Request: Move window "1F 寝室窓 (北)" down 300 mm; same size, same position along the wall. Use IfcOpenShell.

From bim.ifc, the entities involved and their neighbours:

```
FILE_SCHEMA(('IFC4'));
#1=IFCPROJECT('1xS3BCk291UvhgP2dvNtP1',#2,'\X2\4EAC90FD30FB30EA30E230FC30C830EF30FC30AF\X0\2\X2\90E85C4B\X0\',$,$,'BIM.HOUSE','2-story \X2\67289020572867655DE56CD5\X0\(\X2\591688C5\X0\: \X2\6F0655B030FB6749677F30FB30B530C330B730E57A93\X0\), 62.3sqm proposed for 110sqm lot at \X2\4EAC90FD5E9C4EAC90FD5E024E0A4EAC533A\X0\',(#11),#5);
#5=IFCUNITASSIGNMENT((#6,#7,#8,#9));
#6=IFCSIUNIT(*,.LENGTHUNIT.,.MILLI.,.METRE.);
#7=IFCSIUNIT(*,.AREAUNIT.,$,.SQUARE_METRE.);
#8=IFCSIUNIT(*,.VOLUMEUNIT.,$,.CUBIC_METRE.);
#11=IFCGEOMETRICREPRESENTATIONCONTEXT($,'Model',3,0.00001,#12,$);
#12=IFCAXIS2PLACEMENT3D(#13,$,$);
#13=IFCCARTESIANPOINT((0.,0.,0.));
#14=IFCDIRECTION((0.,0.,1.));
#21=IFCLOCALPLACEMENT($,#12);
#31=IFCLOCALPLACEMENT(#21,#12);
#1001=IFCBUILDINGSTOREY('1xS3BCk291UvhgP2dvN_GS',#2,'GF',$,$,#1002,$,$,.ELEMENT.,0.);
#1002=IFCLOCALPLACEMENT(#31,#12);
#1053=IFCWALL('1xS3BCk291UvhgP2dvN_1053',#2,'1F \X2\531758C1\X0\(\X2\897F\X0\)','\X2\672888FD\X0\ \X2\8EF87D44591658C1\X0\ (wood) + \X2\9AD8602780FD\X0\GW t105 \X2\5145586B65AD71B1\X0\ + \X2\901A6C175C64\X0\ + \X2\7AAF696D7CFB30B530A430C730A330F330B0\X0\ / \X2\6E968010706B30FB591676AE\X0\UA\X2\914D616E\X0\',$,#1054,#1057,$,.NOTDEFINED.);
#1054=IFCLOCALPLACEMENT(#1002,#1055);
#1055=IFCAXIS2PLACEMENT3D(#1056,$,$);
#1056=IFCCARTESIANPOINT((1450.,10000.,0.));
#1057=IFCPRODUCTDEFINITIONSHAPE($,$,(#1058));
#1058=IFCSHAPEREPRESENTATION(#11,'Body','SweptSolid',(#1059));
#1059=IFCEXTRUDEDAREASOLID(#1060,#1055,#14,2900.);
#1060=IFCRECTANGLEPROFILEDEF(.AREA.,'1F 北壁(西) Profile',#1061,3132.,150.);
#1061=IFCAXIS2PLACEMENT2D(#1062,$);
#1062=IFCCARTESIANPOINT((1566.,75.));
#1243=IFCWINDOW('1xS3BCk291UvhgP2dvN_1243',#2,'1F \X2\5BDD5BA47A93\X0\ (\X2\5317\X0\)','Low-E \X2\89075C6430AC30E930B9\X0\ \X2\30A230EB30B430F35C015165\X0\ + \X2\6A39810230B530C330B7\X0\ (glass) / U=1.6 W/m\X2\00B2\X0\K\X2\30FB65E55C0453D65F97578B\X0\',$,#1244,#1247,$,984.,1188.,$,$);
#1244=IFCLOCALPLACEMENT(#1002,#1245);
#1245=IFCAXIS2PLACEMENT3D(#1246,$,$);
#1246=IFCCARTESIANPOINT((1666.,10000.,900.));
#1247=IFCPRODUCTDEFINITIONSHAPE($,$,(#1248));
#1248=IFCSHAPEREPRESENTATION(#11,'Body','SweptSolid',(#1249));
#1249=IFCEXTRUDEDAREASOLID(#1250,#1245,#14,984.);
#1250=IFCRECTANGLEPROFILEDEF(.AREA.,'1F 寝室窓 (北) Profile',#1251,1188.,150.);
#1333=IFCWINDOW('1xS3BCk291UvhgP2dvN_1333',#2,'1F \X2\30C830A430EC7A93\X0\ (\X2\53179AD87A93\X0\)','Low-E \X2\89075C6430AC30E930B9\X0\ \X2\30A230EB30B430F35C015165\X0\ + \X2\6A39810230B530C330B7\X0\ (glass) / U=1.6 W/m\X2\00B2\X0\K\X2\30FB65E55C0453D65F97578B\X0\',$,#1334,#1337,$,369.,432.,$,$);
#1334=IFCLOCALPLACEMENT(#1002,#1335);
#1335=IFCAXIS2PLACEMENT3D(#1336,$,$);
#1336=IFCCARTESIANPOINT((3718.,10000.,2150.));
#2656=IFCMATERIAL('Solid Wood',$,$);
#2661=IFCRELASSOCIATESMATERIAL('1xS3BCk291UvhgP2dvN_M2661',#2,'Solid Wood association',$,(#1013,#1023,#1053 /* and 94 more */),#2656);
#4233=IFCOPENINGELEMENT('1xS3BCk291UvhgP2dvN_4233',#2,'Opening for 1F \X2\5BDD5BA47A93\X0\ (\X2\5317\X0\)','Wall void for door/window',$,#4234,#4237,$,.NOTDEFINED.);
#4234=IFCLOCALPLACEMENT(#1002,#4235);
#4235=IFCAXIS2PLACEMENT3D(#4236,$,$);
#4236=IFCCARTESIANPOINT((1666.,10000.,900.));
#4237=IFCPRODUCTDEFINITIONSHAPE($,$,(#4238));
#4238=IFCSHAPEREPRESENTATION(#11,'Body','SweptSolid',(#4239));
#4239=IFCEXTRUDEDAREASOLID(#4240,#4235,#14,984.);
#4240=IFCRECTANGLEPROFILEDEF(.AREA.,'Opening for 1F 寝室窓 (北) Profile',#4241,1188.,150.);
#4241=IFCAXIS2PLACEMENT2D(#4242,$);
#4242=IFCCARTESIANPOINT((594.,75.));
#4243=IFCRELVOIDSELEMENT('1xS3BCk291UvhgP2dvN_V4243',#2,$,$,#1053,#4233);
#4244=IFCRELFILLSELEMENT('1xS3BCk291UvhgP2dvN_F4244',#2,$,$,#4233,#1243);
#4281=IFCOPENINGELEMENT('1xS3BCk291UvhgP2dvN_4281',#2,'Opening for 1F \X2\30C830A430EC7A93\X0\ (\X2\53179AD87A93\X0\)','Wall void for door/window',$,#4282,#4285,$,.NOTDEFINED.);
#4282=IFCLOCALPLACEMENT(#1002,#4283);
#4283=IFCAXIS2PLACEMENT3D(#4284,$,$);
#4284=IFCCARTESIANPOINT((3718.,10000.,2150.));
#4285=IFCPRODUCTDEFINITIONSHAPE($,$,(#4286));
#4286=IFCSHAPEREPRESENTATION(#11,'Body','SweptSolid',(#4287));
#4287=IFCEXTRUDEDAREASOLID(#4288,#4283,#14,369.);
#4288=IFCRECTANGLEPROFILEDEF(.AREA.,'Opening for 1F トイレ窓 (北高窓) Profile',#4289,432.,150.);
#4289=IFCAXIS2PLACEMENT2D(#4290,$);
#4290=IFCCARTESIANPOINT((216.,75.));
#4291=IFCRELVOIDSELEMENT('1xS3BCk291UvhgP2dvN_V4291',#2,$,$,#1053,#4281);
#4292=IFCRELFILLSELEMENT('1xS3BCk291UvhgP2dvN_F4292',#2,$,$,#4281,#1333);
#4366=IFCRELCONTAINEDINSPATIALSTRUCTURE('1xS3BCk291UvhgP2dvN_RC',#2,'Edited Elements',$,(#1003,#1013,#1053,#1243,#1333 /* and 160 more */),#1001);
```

```python
import numpy as np
import ifcopenshell
import ifcopenshell.api.geometry
import ifcopenshell.util.placement
import ifcopenshell.util.unit

model = ifcopenshell.open("bim.ifc")
unit_scale = ifcopenshell.util.unit.calculate_unit_scale(model)

window = model.by_guid("1xS3BCk291UvhgP2dvN_1243")
opening = window.FillsVoids[0].RelatingOpeningElement
dz = -300.0

shift = np.array([0.0, 0.0, dz])
# The window is not placed relative to its opening, so move both.
for product in (opening, window):
    matrix = ifcopenshell.util.placement.get_local_placement(product.ObjectPlacement)
    matrix[:3, 3] += shift
    ifcopenshell.api.geometry.edit_object_placement(model, product=product, matrix=matrix, is_si=False)

print(f"moved by {dz * unit_scale:+.3f} m")

model.write("bim_v2.ifc")
```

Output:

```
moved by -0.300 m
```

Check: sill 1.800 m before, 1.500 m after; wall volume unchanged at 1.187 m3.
